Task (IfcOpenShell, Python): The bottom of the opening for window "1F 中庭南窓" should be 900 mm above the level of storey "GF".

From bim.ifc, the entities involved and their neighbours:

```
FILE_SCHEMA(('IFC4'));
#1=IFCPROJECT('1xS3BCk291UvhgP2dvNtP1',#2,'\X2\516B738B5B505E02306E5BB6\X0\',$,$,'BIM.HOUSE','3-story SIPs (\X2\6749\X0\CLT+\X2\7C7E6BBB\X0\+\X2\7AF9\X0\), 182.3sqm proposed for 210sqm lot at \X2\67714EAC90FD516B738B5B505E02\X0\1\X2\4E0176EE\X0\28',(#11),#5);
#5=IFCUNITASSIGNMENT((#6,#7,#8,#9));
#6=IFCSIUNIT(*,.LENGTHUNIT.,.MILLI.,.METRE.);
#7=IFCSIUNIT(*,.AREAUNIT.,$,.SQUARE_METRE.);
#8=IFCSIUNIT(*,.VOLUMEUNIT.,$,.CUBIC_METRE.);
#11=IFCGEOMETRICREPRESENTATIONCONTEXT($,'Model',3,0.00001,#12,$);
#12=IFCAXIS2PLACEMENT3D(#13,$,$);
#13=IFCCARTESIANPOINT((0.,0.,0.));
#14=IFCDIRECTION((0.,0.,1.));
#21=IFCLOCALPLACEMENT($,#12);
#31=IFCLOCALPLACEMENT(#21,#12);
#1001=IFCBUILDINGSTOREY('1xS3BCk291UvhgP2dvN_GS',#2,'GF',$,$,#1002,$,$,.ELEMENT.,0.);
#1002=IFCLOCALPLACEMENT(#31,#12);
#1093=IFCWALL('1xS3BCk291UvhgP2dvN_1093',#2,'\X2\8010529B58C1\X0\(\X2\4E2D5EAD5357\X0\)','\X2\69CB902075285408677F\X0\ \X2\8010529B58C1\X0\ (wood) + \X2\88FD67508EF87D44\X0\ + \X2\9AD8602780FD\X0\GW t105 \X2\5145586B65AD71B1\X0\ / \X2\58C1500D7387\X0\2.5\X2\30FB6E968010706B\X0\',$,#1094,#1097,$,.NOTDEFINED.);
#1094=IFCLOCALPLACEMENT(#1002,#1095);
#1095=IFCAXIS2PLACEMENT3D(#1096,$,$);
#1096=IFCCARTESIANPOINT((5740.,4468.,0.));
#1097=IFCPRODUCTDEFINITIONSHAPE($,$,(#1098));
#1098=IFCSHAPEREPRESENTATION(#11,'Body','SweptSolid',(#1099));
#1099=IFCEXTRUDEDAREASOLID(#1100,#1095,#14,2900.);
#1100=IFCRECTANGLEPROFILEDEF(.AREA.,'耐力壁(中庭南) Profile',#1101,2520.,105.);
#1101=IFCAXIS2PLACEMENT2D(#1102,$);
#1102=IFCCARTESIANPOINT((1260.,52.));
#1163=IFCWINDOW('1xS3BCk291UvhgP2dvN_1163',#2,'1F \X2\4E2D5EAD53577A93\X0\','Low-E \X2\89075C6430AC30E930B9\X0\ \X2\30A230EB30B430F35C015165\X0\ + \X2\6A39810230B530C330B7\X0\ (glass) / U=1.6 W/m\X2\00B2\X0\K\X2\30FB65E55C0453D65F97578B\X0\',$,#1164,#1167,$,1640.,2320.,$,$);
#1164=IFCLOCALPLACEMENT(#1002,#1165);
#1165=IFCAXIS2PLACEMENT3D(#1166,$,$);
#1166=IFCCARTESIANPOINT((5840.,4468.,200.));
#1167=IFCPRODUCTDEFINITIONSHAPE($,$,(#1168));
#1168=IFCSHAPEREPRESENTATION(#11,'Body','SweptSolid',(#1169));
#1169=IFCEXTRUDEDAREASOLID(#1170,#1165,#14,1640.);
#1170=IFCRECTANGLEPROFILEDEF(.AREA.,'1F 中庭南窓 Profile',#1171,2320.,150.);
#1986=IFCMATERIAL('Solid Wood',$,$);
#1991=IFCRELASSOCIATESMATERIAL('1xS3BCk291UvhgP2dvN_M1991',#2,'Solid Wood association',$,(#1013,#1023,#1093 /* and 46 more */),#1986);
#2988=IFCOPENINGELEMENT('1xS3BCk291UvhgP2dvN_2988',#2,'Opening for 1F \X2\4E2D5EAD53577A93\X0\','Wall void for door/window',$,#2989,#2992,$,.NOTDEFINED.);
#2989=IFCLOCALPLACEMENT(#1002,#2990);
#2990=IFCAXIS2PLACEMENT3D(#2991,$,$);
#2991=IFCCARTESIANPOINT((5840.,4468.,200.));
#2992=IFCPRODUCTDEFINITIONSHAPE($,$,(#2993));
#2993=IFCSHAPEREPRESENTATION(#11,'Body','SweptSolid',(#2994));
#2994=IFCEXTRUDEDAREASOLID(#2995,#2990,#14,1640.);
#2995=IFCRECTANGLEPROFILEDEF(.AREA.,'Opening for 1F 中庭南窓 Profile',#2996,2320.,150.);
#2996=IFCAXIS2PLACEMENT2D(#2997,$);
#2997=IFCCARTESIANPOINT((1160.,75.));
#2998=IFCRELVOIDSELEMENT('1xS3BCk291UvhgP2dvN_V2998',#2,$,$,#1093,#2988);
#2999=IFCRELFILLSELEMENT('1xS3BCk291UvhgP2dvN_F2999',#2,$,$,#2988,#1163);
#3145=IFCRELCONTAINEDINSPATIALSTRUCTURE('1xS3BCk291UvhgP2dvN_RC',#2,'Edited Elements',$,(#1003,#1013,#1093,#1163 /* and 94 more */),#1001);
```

```python
import numpy as np
import ifcopenshell
import ifcopenshell.api.geometry
import ifcopenshell.geom
import ifcopenshell.util.element
import ifcopenshell.util.placement
import ifcopenshell.util.shape
import ifcopenshell.util.unit

model = ifcopenshell.open("bim.ifc")
unit_scale = ifcopenshell.util.unit.calculate_unit_scale(model)

window = model.by_guid("1xS3BCk291UvhgP2dvN_1163")
opening = window.FillsVoids[0].RelatingOpeningElement
storey = ifcopenshell.util.element.get_container(window, ifc_class="IfcBuildingStorey")
level = ifcopenshell.util.placement.get_local_placement(storey.ObjectPlacement)[2, 3]

# The opening's origin need not be at the sill, so measure its lowest point.
shape = ifcopenshell.geom.create_shape(ifcopenshell.geom.settings(), opening)
bottom = ifcopenshell.util.shape.get_shape_bottom_elevation(shape, shape.geometry) / unit_scale
dz = level + 0.9 / unit_scale - bottom

shift = np.array([0.0, 0.0, dz])
# The window is not placed relative to its opening, so move both.
for product in (opening, window):
    matrix = ifcopenshell.util.placement.get_local_placement(product.ObjectPlacement)
    matrix[:3, 3] += shift
    ifcopenshell.api.geometry.edit_object_placement(model, product=product, matrix=matrix, is_si=False)

print(f"moved by {dz * unit_scale:+.3f} m")

model.write("bim-out.ifc")
```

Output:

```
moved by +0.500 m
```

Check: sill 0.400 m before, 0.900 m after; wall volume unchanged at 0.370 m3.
